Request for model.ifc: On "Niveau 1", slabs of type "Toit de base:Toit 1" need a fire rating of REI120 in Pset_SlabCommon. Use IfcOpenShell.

First a look at what the model holds.

```python
import ifcopenshell
import ifcopenshell.util.element

model = ifcopenshell.open("model.ifc")
print(model.schema)
storey = next(s for s in model.by_type("IfcBuildingStorey") if s.Name == "Niveau 1")
slabs = [e for e in ifcopenshell.util.element.get_decomposition(storey) if e.is_a("IfcSlab")]
seen = {}
for e in slabs:
    element_type = ifcopenshell.util.element.get_type(e)
    key = (element_type.Name if element_type != e and element_type else None, ifcopenshell.util.element.get_pset(e, "Pset_SlabCommon", "FireRating"))
    seen[key] = seen.get(key, 0) + 1
for (name, value), count in sorted(seen.items(), key=str):
    print(count, "x", name, "|", value)
```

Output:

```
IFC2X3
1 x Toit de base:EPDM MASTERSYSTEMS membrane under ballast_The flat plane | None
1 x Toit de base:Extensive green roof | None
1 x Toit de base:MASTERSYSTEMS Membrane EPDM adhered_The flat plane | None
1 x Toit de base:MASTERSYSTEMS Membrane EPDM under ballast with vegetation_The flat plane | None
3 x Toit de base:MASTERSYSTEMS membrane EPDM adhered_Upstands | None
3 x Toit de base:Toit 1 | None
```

```python
import ifcopenshell
import ifcopenshell.api.pset
import ifcopenshell.util.element

model = ifcopenshell.open("model.ifc")

storey = next(s for s in model.by_type("IfcBuildingStorey") if s.Name == "Niveau 1")
slabs = [e for e in ifcopenshell.util.element.get_decomposition(storey) if e.is_a("IfcSlab")]

count = 0
for e in slabs:
    element_type = ifcopenshell.util.element.get_type(e)
    if element_type in (None, e) or element_type.Name != "Toit de base:Toit 1":
        continue
    # add_pset returns the element's existing set when there is one.
    pset = ifcopenshell.api.pset.add_pset(model, product=e, name="Pset_SlabCommon")
    ifcopenshell.api.pset.edit_pset(model, pset=pset, properties={"FireRating": "REI120"})
    count += 1

print(count, "slabs updated")

model.write("model_updated.ifc")
```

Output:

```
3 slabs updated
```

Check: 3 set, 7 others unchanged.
